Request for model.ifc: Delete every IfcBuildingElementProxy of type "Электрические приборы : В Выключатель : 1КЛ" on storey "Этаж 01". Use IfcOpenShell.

First a look at what the model holds.

```python
import ifcopenshell
import ifcopenshell.util.element

model = ifcopenshell.open("model.ifc")
print(model.schema)
storey = next(s for s in model.by_type("IfcBuildingStorey") if s.Name == "Этаж 01")
proxies = [e for e in ifcopenshell.util.element.get_decomposition(storey) if e.is_a("IfcBuildingElementProxy")]
seen = {}
for e in proxies:
    element_type = ifcopenshell.util.element.get_type(e)
    name = element_type.Name if element_type not in (None, e) else None
    seen[name] = seen.get(name, 0) + 1
for name, count in sorted(seen.items(), key=str):
    print(count, "x", name)
```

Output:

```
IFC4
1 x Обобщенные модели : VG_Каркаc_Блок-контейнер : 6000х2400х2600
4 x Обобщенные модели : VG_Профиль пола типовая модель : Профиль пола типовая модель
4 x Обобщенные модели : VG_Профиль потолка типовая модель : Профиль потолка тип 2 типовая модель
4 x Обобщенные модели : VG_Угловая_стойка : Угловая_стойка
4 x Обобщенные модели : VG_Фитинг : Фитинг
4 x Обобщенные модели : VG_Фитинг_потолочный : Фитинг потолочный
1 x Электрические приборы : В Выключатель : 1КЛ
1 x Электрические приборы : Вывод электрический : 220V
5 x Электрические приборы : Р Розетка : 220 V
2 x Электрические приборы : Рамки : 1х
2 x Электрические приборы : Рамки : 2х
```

```python
import ifcopenshell
import ifcopenshell.api.root
import ifcopenshell.util.element

model = ifcopenshell.open("model.ifc")

storey = next(s for s in model.by_type("IfcBuildingStorey") if s.Name == "Этаж 01")
proxies = [e for e in ifcopenshell.util.element.get_decomposition(storey) if e.is_a("IfcBuildingElementProxy")]
targets = [e for e in proxies if (t := ifcopenshell.util.element.get_type(e)) not in (None, e) and t.Name == "Электрические приборы : В Выключатель : 1КЛ"]

for e in targets:
    ifcopenshell.api.root.remove_product(model, product=e)
print(len(targets), "removed")

model.write("model_updated.ifc")
```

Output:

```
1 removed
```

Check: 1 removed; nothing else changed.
